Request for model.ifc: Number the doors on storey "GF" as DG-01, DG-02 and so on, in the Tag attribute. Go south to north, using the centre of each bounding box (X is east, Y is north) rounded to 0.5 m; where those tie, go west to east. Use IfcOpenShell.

First a look at what the model holds.

```python
import ifcopenshell
import ifcopenshell.util.element
import ifcopenshell.util.placement

model = ifcopenshell.open("model.ifc")
print(model.schema)
storey = next(s for s in model.by_type("IfcBuildingStorey") if s.Name == "GF")
doors = [e for e in ifcopenshell.util.element.get_decomposition(storey) if e.is_a("IfcDoor")]
for e in sorted(doors, key=lambda e: e.id()):
    origin = ifcopenshell.util.placement.get_local_placement(e.ObjectPlacement)[:3, 3]
    print(e.id(), e.Tag, e.Name, origin.round(2) + 0.0, sep=" | ")
```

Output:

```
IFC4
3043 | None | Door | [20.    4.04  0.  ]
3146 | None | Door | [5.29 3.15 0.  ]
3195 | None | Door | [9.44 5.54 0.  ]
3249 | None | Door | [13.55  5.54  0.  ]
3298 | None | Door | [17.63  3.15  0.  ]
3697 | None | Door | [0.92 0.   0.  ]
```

```python
import ifcopenshell
import ifcopenshell.geom
import ifcopenshell.util.element
import ifcopenshell.util.shape

model = ifcopenshell.open("model.ifc")
settings = ifcopenshell.geom.settings()
settings.set("use-world-coords", True)


def centre(element):
    shape = ifcopenshell.geom.create_shape(settings, element)
    return ifcopenshell.util.shape.get_bbox_centroid(shape.geometry)


storey = next(s for s in model.by_type("IfcBuildingStorey") if s.Name == "GF")
doors = [e for e in ifcopenshell.util.element.get_decomposition(storey) if e.is_a("IfcDoor")]

# Insertion points can sit at a corner or the storey origin, so sort by the geometry (in metres).
centres = {e: centre(e) for e in doors}
doors.sort(key=lambda e: (round(centres[e][1] / 0.5), centres[e][0]))

for i, e in enumerate(doors, start=1):
    number = f"DG-{i:02d}"
    e.Tag = number
    print(e.id(), number)

model.write("model_rev.ifc")
```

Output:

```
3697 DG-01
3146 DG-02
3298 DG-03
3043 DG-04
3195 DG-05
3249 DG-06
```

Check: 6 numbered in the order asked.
